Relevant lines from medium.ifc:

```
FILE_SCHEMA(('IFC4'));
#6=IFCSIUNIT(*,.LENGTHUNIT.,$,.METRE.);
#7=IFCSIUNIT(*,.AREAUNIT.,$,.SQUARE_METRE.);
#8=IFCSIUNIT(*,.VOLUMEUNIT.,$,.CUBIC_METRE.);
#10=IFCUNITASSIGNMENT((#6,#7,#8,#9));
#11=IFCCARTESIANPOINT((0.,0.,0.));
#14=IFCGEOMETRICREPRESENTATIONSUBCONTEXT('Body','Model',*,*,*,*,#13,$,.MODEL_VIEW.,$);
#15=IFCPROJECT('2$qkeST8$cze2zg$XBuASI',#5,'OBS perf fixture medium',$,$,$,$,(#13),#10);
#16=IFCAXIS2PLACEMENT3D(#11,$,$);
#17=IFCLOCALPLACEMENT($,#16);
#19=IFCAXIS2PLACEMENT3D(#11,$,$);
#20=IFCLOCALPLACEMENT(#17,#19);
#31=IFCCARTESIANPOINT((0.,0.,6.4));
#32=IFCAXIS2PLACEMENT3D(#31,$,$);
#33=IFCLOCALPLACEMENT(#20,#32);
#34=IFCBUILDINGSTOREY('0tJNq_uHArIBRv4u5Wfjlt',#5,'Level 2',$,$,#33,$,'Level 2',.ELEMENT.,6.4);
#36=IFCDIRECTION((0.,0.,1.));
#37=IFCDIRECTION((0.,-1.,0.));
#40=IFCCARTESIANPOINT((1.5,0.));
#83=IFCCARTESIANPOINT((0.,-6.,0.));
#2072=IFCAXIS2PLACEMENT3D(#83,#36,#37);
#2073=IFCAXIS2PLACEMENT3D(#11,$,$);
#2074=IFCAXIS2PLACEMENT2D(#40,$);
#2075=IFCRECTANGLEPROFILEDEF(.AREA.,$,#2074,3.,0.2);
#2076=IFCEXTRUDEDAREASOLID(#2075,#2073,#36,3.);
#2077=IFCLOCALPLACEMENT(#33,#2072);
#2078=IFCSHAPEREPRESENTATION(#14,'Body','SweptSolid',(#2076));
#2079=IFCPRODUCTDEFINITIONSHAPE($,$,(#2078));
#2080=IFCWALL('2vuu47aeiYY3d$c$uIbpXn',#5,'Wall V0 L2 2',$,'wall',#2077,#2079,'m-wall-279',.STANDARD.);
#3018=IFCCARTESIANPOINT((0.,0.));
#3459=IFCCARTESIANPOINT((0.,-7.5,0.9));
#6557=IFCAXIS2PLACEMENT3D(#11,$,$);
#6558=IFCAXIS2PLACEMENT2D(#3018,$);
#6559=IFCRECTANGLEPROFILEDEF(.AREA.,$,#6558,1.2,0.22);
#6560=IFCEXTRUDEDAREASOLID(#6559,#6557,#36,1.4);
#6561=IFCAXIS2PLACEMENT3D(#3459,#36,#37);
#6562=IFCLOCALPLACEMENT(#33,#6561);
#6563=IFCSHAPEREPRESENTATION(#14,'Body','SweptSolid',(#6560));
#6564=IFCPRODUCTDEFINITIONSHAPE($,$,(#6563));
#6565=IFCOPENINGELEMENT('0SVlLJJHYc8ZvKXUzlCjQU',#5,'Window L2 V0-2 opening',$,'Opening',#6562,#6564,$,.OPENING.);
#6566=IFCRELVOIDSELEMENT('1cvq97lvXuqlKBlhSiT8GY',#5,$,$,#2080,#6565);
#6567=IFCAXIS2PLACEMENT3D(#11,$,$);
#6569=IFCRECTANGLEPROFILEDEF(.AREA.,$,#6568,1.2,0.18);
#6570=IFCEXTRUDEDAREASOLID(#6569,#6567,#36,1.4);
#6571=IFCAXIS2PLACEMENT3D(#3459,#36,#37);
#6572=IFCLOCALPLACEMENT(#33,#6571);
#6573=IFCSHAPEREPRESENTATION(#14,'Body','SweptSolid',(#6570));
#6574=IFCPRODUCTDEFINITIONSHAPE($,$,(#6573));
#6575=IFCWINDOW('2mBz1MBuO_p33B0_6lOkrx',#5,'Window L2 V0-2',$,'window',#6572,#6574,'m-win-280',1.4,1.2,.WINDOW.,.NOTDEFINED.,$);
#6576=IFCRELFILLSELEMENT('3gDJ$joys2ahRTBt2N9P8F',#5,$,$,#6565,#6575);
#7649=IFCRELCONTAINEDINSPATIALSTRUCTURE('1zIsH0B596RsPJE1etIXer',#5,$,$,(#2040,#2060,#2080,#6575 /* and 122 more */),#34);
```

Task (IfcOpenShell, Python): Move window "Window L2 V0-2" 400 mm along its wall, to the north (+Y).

```python
import ifcopenshell
import ifcopenshell.api.geometry
import ifcopenshell.util.placement
import ifcopenshell.util.unit

model = ifcopenshell.open("medium.ifc")
unit_scale = ifcopenshell.util.unit.calculate_unit_scale(model)

window = model.by_id(6575)
opening = window.FillsVoids[0].RelatingOpeningElement
wall = opening.VoidsElements[0].RelatingBuildingElement

wall_matrix = ifcopenshell.util.placement.get_local_placement(wall.ObjectPlacement)
shift = wall_matrix[:3, 0] * -0.4 / unit_scale
before = ifcopenshell.util.placement.get_local_placement(window.ObjectPlacement)[:3, 3].copy()

# The window is not placed relative to its opening, so move both.
for product in (opening, window):
    matrix = ifcopenshell.util.placement.get_local_placement(product.ObjectPlacement)
    matrix[:3, 3] += shift
    ifcopenshell.api.geometry.edit_object_placement(model, product=product, matrix=matrix, is_si=False)

after = ifcopenshell.util.placement.get_local_placement(window.ObjectPlacement)[:3, 3]
print("window moved by", (after - before).round(3) + 0.0)

model.write("medium-out.ifc")
```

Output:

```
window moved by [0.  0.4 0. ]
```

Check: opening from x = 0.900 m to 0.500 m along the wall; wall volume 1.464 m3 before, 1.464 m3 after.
